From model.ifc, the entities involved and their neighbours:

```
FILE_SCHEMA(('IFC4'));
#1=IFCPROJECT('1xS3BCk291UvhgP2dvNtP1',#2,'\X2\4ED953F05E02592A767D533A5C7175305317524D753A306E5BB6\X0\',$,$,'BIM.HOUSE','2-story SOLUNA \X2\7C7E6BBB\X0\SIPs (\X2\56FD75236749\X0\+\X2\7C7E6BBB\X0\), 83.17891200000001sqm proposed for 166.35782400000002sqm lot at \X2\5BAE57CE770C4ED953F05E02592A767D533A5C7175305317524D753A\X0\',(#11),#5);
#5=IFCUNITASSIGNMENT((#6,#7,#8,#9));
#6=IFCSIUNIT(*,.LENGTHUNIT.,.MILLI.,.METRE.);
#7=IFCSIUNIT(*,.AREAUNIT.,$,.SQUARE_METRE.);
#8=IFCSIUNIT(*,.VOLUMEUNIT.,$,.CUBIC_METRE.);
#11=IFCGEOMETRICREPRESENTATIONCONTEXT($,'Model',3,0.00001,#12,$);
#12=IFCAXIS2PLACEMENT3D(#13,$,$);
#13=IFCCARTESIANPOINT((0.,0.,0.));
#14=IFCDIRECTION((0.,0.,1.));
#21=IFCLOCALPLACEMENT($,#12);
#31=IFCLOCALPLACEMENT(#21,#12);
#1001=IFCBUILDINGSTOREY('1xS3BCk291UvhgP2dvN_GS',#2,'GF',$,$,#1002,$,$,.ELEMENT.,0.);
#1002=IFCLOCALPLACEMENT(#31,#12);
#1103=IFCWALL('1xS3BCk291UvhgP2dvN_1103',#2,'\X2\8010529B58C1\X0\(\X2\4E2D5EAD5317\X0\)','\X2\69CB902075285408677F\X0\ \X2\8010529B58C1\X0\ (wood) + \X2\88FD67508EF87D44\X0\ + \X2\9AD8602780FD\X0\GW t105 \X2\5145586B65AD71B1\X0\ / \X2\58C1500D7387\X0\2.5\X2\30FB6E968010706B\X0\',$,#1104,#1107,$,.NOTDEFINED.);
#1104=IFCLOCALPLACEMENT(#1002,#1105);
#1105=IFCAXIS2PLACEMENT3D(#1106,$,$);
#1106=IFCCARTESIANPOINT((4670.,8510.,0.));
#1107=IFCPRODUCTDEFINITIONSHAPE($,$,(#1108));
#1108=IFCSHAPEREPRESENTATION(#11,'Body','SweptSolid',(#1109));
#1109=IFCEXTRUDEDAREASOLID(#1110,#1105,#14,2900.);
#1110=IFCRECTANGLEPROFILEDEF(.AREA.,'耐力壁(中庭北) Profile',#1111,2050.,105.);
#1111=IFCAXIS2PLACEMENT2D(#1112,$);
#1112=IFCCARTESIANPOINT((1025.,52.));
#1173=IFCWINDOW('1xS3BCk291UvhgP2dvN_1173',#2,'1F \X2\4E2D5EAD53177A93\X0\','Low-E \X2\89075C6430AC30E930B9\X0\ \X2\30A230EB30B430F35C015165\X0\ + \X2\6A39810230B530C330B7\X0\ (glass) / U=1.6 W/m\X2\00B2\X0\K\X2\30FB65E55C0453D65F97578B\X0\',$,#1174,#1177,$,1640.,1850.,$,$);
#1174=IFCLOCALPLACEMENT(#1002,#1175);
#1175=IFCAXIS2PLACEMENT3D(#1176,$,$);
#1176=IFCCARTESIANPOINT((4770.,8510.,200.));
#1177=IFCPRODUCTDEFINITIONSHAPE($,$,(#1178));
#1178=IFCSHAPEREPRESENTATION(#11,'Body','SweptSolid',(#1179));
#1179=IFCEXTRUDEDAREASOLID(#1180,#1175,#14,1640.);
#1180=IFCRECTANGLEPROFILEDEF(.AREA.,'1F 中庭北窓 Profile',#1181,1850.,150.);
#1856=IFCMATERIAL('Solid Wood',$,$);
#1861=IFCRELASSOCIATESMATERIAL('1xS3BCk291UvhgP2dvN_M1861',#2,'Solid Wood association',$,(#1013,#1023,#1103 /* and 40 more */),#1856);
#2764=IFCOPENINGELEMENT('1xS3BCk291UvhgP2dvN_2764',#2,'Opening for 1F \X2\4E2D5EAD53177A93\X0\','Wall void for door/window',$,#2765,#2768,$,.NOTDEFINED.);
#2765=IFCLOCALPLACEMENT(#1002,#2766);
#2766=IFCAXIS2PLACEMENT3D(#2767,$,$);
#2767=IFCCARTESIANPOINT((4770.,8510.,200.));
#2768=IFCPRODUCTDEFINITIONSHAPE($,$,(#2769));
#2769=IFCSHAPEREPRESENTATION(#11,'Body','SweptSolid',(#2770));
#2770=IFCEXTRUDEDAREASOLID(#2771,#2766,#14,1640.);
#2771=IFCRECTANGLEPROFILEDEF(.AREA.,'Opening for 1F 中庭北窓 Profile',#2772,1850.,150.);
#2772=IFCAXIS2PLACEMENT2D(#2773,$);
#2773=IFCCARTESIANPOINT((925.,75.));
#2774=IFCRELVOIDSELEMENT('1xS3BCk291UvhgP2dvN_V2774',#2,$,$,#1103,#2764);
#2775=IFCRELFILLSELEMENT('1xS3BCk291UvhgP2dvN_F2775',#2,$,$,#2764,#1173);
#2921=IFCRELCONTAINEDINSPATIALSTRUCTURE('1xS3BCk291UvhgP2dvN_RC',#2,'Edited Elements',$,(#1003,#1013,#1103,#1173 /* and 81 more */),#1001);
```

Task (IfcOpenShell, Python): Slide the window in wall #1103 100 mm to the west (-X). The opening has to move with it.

```python
import ifcopenshell
import ifcopenshell.api.geometry
import ifcopenshell.util.placement
import ifcopenshell.util.unit

model = ifcopenshell.open("model.ifc")
unit_scale = ifcopenshell.util.unit.calculate_unit_scale(model)

window = model.by_guid("1xS3BCk291UvhgP2dvN_1173")
opening = window.FillsVoids[0].RelatingOpeningElement
wall = opening.VoidsElements[0].RelatingBuildingElement

wall_matrix = ifcopenshell.util.placement.get_local_placement(wall.ObjectPlacement)
shift = wall_matrix[:3, 0] * -0.1 / unit_scale
before = ifcopenshell.util.placement.get_local_placement(window.ObjectPlacement)[:3, 3].copy()

# The window is not placed relative to its opening, so move both.
for product in (opening, window):
    matrix = ifcopenshell.util.placement.get_local_placement(product.ObjectPlacement)
    matrix[:3, 3] += shift
    ifcopenshell.api.geometry.edit_object_placement(model, product=product, matrix=matrix, is_si=False)

after = ifcopenshell.util.placement.get_local_placement(window.ObjectPlacement)[:3, 3]
print("window moved by", (after - before).round(3) + 0.0)

model.write("model_edited.ifc")
```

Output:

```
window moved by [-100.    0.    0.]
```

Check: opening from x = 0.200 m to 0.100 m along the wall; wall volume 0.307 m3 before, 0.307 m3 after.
